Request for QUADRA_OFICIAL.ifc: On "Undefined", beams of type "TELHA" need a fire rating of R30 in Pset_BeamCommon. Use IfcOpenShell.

First a look at what the model holds.

```python
import ifcopenshell
import ifcopenshell.util.element

model = ifcopenshell.open("QUADRA_OFICIAL.ifc")
print(model.schema)
storey = next(s for s in model.by_type("IfcBuildingStorey") if s.Name == "Undefined")
beams = [e for e in ifcopenshell.util.element.get_decomposition(storey) if e.is_a("IfcBeam")]
seen = {}
for e in beams:
    element_type = ifcopenshell.util.element.get_type(e)
    key = (element_type.Name if element_type != e and element_type else None, ifcopenshell.util.element.get_pset(e, "Pset_BeamCommon", "FireRating"))
    seen[key] = seen.get(key, 0) + 1
for (name, value), count in sorted(seen.items(), key=str):
    print(count, "x", name, "|", value)
```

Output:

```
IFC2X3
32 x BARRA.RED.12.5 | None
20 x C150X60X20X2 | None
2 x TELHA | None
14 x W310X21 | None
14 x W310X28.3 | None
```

```python
import ifcopenshell
import ifcopenshell.api.pset
import ifcopenshell.util.element

model = ifcopenshell.open("QUADRA_OFICIAL.ifc")

storey = next(s for s in model.by_type("IfcBuildingStorey") if s.Name == "Undefined")
beams = [e for e in ifcopenshell.util.element.get_decomposition(storey) if e.is_a("IfcBeam")]

count = 0
for e in beams:
    element_type = ifcopenshell.util.element.get_type(e)
    if element_type in (None, e) or element_type.Name != "TELHA":
        continue
    found = ifcopenshell.util.element.get_pset(e, "Pset_BeamCommon", should_inherit=False)
    if found:
        pset = model.by_id(found["id"])
        if len(ifcopenshell.util.element.get_elements_by_pset(pset)) > 1:
            pset = ifcopenshell.api.pset.unshare_pset(model, products=[e], pset=pset)[0]
    else:
        pset = ifcopenshell.api.pset.add_pset(model, product=e, name="Pset_BeamCommon")
    ifcopenshell.api.pset.edit_pset(model, pset=pset, properties={"FireRating": "R30"})
    count += 1

print(count, "beams updated")

model.write("QUADRA_OFICIAL-out.ifc")
```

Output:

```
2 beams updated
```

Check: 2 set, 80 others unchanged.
